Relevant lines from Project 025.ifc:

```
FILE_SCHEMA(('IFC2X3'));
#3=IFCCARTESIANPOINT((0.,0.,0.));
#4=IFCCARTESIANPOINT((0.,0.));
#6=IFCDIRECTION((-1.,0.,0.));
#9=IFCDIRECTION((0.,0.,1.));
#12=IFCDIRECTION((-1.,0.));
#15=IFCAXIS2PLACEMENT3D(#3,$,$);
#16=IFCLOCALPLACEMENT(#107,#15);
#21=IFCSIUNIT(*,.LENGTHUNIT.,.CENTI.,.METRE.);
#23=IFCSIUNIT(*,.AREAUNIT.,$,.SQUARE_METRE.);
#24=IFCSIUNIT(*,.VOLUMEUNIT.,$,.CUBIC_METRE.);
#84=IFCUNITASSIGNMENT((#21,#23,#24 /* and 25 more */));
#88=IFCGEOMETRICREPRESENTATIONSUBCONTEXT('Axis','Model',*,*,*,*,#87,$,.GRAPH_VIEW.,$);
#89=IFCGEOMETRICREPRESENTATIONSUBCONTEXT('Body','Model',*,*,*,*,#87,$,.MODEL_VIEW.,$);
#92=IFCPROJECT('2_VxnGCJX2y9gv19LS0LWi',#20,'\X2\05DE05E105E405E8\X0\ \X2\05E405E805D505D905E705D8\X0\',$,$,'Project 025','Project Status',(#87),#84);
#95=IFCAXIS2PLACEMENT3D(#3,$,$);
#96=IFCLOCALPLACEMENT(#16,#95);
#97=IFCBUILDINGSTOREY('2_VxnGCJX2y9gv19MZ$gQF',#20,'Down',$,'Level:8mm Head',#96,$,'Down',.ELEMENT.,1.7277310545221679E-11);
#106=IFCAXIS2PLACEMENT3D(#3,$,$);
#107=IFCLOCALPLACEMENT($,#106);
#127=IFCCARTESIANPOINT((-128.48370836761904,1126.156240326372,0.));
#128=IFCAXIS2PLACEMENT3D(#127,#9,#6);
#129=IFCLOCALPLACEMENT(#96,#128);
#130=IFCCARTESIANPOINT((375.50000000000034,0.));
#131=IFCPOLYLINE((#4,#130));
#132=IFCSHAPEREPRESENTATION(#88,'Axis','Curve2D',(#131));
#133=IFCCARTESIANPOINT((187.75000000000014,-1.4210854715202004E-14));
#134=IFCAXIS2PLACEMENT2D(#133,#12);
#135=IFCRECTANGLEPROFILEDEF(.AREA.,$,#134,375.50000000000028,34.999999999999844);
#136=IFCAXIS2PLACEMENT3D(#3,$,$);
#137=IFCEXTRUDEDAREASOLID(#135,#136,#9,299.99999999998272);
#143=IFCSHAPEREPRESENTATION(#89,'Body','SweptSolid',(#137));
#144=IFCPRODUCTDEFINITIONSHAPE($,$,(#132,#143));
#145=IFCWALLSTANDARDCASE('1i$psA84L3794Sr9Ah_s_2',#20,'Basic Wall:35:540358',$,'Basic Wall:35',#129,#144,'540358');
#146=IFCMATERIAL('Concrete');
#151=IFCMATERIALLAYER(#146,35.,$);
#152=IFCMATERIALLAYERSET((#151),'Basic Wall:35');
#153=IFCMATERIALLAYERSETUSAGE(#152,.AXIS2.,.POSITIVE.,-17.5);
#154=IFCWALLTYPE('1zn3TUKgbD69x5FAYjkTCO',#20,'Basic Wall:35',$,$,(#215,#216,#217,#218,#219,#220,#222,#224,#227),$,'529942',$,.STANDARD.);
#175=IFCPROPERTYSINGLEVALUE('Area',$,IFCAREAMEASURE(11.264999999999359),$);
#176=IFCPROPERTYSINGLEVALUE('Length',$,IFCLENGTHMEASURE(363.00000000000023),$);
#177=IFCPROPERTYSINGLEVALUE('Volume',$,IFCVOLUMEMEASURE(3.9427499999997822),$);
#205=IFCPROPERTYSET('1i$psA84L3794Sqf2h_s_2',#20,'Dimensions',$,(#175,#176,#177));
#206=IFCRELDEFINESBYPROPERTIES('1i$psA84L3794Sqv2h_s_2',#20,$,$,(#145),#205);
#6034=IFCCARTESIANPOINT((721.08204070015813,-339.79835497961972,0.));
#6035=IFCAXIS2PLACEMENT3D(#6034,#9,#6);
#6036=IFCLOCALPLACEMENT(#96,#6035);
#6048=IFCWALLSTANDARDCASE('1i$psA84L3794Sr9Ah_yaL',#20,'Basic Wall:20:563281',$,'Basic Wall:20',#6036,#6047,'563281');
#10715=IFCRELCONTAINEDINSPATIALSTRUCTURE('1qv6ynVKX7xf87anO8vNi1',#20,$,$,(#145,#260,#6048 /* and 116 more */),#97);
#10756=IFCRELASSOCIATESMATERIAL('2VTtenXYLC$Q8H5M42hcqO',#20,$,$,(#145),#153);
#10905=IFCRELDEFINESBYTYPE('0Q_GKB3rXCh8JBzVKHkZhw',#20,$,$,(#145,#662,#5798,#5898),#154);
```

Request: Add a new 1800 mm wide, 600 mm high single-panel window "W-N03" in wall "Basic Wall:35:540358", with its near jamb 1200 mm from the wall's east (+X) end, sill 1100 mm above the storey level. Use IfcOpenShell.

```python
import numpy as np
import ifcopenshell
import ifcopenshell.api.feature
import ifcopenshell.api.geometry
import ifcopenshell.api.pset
import ifcopenshell.api.root
import ifcopenshell.api.spatial
import ifcopenshell.api.type
import ifcopenshell.geom
import ifcopenshell.util.element
import ifcopenshell.util.placement
import ifcopenshell.util.representation
import ifcopenshell.util.shape
import ifcopenshell.util.unit

model = ifcopenshell.open("Project 025.ifc")
unit_scale = ifcopenshell.util.unit.calculate_unit_scale(model)
area_scale = ifcopenshell.util.unit.calculate_unit_scale(model, "AREAUNIT")
volume_scale = ifcopenshell.util.unit.calculate_unit_scale(model, "VOLUMEUNIT")
settings = ifcopenshell.geom.settings()


def volume(element):
    """Net volume in cubic metres, openings subtracted."""
    shape = ifcopenshell.geom.create_shape(settings, element)
    return ifcopenshell.util.shape.get_volume(shape.geometry)


wall = model.by_id(145)
storey = ifcopenshell.util.element.get_container(wall, ifc_class="IfcBuildingStorey")
context = ifcopenshell.util.representation.get_context(model, "Model", "Body", "MODEL_VIEW")
before = volume(wall)

width, height, from_end, sill = 1.8, 0.6, 1.2, 1.1  # metres

# The wall runs along its own X axis, and the end named is its -X end.
wall_shape = ifcopenshell.geom.create_shape(settings, wall)
x, y, z = ifcopenshell.util.shape.get_vertices(wall_shape.geometry).T
start = x.min() + from_end
face, thickness = float(y.min()), float(y.max() - y.min())
wall_matrix = ifcopenshell.util.placement.get_local_placement(wall.ObjectPlacement)
level = ifcopenshell.util.placement.get_local_placement(storey.ObjectPlacement)[2, 3]


def in_wall(x, y):
    """Placement at x, y metres in the wall's axes, at sill height."""
    matrix = wall_matrix.copy()
    matrix[:, 3] = wall_matrix @ np.array([x / unit_scale, y / unit_scale, 0.0, 1.0])
    matrix[2, 3] = level + sill / unit_scale
    return matrix


# Opening: a box that overshoots both wall faces by 50 mm.
opening = ifcopenshell.api.root.create_entity(model, ifc_class="IfcOpeningElement")
box = ifcopenshell.api.geometry.add_wall_representation(
    model, context=context, length=width, height=height, thickness=thickness + 0.1
)
ifcopenshell.api.geometry.assign_representation(model, product=opening, representation=box)
ifcopenshell.api.geometry.edit_object_placement(model, product=opening, matrix=in_wall(start, face - 0.05), is_si=False)
ifcopenshell.api.feature.add_feature(model, feature=opening, element=wall)

window = ifcopenshell.api.root.create_entity(model, ifc_class="IfcWindow", name="W-N03")
window.OverallWidth, window.OverallHeight = width / unit_scale, height / unit_scale
body = ifcopenshell.api.geometry.add_window_representation(
    model,
    context=context,
    overall_width=window.OverallWidth,
    overall_height=window.OverallHeight,
    partition_type="SINGLE_PANEL",
)
ifcopenshell.api.geometry.assign_representation(model, product=window, representation=body)
ifcopenshell.api.spatial.assign_container(model, products=[window], relating_structure=storey)
fills = ifcopenshell.api.feature.add_filling(model, opening=opening, element=window)
fills.OwnerHistory = window.OwnerHistory  # required in IFC2X3

# IFC2X3 keeps the operation on the window style.
style = ifcopenshell.api.root.create_entity(model, ifc_class="IfcWindowStyle", name="W-N03")
style.OperationType, style.ConstructionType = "SINGLE_PANEL", "NOTDEFINED"
style.ParameterTakesPrecedence = style.Sizeable = False
ifcopenshell.api.type.assign_type(model, related_objects=[window], relating_type=style)

# Centre the window in the wall's thickness.
ifcopenshell.api.geometry.edit_object_placement(model, product=window, matrix=in_wall(start, face), is_si=False)
window_shape = ifcopenshell.geom.create_shape(settings, window)
depth = ifcopenshell.util.shape.get_vertices(window_shape.geometry)[:, 1]
offset = face + thickness / 2 - (depth.min() + depth.max()) / 2
ifcopenshell.api.geometry.edit_object_placement(model, product=window, matrix=in_wall(start, offset), is_si=False)

after = volume(wall)

# Update the wall's stored quantities.
pset = model.by_id(ifcopenshell.util.element.get_pset(wall, "Dimensions", should_inherit=False)["id"])
ifcopenshell.api.pset.edit_pset(model, pset=pset, properties={
    "Area": model.create_entity("IfcAreaMeasure", after / thickness / area_scale),
    "Volume": model.create_entity("IfcVolumeMeasure", after / volume_scale),
})

print(f"wall volume {before:.3f} -> {after:.3f} m3")

model.write("Project 025_edited.ifc")
```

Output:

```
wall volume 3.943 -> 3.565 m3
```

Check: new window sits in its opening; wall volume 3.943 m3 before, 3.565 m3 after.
